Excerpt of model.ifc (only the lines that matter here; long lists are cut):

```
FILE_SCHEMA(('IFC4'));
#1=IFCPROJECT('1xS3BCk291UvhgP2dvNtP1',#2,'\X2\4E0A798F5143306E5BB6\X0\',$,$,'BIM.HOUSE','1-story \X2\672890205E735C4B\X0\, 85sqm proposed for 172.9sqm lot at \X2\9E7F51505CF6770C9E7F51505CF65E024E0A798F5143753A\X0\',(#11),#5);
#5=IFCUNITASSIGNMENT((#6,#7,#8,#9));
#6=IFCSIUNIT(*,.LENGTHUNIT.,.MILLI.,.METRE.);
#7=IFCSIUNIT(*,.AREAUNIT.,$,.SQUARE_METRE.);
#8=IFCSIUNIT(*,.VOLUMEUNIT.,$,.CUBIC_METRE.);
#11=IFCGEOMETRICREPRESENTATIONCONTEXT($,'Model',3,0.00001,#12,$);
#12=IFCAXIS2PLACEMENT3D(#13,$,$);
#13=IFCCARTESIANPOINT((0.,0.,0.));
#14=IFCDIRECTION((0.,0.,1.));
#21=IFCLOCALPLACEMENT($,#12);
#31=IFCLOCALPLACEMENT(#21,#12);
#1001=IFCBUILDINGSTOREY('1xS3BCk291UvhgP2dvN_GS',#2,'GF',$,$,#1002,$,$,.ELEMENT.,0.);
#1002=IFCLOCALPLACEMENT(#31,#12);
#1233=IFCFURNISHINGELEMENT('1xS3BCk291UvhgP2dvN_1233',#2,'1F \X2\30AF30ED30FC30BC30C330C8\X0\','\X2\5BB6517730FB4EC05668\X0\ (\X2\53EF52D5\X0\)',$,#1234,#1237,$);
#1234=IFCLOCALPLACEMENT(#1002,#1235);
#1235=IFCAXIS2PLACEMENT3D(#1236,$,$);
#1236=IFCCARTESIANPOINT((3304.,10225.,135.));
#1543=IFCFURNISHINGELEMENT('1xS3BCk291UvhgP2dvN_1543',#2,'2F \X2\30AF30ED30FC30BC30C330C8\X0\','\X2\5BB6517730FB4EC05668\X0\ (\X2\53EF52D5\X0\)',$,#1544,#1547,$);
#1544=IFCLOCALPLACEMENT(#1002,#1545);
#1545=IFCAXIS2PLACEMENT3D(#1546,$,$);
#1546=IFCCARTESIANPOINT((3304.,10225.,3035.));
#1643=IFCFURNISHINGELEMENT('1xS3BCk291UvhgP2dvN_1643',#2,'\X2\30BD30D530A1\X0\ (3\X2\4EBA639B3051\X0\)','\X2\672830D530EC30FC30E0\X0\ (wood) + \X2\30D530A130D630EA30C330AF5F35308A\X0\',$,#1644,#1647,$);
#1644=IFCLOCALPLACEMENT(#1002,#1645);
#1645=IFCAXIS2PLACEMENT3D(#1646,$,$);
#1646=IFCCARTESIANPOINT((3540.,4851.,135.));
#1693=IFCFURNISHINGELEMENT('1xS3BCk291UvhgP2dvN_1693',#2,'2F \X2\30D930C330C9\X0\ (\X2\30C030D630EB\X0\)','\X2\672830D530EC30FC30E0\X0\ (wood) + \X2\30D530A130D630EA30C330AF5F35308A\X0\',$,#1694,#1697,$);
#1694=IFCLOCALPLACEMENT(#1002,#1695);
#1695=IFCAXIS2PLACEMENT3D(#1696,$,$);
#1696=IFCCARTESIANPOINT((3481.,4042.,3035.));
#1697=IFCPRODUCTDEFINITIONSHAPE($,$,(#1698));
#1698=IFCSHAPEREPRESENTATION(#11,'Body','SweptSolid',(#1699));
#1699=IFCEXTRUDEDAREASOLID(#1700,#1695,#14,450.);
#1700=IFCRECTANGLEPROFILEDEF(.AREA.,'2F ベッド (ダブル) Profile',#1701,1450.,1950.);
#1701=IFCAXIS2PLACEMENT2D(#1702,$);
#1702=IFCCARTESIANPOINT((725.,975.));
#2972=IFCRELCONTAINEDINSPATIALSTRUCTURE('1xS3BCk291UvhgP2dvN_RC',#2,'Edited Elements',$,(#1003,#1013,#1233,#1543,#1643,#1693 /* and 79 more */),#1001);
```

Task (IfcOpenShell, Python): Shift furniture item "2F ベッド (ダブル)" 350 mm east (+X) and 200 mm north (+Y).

```python
import ifcopenshell
import ifcopenshell.api.geometry
import ifcopenshell.util.placement
import ifcopenshell.util.unit

model = ifcopenshell.open("model.ifc")
unit_scale = ifcopenshell.util.unit.calculate_unit_scale(model)

item = model.by_guid("1xS3BCk291UvhgP2dvN_1693")
matrix = ifcopenshell.util.placement.get_local_placement(item.ObjectPlacement)
matrix[0, 3] += 0.35 / unit_scale
matrix[1, 3] += 0.2 / unit_scale
ifcopenshell.api.geometry.edit_object_placement(model, product=item, matrix=matrix, is_si=False)

print(ifcopenshell.util.placement.get_local_placement(item.ObjectPlacement).round(3) + 0.0)

model.write("model_v2.ifc")
```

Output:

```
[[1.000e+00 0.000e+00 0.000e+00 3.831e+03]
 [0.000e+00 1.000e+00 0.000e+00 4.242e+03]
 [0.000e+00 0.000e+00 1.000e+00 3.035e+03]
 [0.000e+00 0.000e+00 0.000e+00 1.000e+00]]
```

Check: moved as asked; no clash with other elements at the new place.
